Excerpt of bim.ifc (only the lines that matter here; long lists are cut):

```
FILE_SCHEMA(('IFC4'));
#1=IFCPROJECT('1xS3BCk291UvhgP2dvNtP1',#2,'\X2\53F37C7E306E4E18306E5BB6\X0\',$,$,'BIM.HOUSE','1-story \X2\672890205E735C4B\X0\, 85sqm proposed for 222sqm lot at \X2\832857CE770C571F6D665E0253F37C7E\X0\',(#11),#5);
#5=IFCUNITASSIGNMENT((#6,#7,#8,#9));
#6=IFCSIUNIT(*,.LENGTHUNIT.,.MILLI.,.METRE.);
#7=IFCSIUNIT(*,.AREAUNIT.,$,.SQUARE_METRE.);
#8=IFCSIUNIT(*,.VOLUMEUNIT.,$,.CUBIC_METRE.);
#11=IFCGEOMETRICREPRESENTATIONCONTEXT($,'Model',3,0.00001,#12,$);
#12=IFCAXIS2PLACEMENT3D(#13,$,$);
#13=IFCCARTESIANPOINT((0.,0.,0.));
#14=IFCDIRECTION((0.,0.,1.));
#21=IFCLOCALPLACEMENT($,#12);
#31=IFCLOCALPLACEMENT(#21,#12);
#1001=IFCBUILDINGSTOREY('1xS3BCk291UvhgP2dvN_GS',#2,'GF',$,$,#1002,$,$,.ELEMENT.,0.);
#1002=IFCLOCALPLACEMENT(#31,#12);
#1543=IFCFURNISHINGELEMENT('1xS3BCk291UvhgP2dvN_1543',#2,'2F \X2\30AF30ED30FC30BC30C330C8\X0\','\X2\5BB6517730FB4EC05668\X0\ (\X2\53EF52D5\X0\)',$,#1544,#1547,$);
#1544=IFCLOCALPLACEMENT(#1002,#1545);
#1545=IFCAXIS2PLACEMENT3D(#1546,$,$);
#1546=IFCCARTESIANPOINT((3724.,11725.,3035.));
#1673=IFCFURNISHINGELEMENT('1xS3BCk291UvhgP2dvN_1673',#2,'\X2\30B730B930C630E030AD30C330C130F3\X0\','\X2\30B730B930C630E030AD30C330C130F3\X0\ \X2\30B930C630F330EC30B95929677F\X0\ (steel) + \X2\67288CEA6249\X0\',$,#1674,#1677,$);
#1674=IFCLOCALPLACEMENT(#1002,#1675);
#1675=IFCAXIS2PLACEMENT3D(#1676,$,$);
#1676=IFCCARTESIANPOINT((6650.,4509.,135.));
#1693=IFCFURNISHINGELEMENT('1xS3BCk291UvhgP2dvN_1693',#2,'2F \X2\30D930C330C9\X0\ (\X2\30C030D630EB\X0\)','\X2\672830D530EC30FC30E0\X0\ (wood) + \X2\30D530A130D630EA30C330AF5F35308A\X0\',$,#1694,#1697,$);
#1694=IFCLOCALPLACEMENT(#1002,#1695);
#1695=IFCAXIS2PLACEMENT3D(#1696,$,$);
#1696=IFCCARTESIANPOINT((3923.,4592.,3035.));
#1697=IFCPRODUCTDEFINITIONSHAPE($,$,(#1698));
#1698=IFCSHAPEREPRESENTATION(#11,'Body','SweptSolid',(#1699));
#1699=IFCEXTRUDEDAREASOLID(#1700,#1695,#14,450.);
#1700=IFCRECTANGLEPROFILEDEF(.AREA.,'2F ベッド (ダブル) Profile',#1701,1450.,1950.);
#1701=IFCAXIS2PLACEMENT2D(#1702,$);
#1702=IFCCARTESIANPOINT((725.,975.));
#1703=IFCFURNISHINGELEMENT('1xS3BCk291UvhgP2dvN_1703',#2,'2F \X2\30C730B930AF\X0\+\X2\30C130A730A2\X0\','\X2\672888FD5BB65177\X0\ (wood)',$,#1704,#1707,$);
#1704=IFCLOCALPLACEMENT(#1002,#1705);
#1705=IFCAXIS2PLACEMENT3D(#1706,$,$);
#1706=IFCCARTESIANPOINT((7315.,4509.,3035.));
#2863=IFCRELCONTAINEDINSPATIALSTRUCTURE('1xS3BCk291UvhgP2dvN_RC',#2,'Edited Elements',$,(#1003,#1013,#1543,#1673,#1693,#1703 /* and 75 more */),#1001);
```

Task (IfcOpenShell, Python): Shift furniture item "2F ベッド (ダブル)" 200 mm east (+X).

```python
import ifcopenshell
import ifcopenshell.api.geometry
import ifcopenshell.util.placement

model = ifcopenshell.open("bim.ifc")

item = model.by_guid("1xS3BCk291UvhgP2dvN_1693")
matrix = ifcopenshell.util.placement.get_local_placement(item.ObjectPlacement)
matrix[0, 3] += 200.0
ifcopenshell.api.geometry.edit_object_placement(model, product=item, matrix=matrix, is_si=False)

print(ifcopenshell.util.placement.get_local_placement(item.ObjectPlacement).round(3) + 0.0)

model.write("bim_edited.ifc")
```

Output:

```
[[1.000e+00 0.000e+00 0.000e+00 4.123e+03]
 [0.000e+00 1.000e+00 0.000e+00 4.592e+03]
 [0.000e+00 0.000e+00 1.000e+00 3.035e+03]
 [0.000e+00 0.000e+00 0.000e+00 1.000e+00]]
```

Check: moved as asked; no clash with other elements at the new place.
